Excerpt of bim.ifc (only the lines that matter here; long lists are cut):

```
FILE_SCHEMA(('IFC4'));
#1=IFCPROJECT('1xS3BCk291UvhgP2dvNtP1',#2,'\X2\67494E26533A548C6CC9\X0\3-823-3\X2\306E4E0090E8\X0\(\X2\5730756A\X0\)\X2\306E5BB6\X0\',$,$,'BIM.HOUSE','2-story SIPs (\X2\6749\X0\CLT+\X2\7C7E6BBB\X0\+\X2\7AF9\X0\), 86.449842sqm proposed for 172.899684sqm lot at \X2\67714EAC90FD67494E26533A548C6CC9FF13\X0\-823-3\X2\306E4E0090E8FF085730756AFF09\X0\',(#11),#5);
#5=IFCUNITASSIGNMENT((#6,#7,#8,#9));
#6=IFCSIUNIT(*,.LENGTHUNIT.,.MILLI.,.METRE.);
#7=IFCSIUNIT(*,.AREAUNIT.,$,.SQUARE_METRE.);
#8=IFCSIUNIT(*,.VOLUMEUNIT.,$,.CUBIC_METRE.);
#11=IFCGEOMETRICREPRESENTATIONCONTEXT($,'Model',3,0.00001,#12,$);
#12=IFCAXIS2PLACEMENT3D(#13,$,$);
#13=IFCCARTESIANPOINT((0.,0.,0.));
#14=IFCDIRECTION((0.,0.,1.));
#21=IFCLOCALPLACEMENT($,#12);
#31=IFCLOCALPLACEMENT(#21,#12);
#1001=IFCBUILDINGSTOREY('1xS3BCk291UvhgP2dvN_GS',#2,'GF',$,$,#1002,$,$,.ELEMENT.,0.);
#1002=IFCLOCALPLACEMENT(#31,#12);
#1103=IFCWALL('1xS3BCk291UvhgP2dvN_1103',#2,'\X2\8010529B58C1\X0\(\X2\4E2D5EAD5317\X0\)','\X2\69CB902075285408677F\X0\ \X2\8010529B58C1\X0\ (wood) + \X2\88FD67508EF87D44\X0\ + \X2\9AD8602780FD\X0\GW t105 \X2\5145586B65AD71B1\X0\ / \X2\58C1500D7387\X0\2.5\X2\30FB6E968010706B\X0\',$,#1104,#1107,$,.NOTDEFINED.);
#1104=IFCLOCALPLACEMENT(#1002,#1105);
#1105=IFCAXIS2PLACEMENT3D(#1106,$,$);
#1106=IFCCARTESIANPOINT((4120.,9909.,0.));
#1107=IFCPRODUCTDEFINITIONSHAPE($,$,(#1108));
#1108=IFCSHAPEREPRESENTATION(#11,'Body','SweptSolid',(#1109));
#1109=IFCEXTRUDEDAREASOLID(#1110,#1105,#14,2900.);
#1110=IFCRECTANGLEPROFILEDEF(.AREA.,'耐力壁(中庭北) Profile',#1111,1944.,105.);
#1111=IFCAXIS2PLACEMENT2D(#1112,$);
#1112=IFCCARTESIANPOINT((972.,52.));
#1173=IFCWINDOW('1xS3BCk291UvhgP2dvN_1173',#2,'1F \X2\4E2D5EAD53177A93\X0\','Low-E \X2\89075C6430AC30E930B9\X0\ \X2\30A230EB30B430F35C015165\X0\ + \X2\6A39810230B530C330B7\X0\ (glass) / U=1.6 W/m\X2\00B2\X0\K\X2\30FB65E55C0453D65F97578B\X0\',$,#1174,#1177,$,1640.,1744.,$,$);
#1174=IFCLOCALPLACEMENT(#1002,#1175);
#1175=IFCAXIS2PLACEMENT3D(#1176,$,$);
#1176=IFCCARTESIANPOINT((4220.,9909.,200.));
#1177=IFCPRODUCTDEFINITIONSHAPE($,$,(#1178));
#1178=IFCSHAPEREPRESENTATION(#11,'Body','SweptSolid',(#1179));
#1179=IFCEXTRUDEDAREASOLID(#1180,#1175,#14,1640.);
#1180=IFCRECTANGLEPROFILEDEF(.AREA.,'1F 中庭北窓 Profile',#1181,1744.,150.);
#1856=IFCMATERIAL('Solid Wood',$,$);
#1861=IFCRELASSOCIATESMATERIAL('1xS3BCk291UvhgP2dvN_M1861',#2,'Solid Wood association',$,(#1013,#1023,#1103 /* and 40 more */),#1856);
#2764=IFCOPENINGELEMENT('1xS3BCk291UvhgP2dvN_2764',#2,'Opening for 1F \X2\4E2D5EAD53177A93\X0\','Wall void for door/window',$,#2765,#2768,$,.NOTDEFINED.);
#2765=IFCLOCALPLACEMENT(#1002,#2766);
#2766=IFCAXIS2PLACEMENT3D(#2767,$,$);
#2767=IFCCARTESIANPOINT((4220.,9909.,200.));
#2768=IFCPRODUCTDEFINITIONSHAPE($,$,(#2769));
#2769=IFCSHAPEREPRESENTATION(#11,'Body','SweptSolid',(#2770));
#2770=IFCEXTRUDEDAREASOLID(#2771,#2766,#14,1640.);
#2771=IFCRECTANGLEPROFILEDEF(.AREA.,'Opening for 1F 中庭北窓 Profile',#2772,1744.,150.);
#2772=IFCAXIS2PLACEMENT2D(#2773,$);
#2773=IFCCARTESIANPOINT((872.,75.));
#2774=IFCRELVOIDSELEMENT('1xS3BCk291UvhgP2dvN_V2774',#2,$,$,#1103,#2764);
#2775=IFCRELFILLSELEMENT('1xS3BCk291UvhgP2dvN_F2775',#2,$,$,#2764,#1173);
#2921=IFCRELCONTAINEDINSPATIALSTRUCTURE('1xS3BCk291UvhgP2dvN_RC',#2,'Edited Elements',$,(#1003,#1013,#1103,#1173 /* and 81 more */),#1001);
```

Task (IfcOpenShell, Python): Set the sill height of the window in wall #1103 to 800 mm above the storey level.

```python
import numpy as np
import ifcopenshell
import ifcopenshell.api.geometry
import ifcopenshell.geom
import ifcopenshell.util.element
import ifcopenshell.util.placement
import ifcopenshell.util.shape
import ifcopenshell.util.unit

model = ifcopenshell.open("bim.ifc")
unit_scale = ifcopenshell.util.unit.calculate_unit_scale(model)

window = model.by_guid("1xS3BCk291UvhgP2dvN_1173")
opening = window.FillsVoids[0].RelatingOpeningElement
storey = ifcopenshell.util.element.get_container(window, ifc_class="IfcBuildingStorey")
level = ifcopenshell.util.placement.get_local_placement(storey.ObjectPlacement)[2, 3]

# The opening's origin need not be at the sill, so measure its lowest point.
shape = ifcopenshell.geom.create_shape(ifcopenshell.geom.settings(), opening)
bottom = ifcopenshell.util.shape.get_shape_bottom_elevation(shape, shape.geometry) / unit_scale
dz = level + 0.8 / unit_scale - bottom

shift = np.array([0.0, 0.0, dz])
# The window is not placed relative to its opening, so move both.
for product in (opening, window):
    matrix = ifcopenshell.util.placement.get_local_placement(product.ObjectPlacement)
    matrix[:3, 3] += shift
    ifcopenshell.api.geometry.edit_object_placement(model, product=product, matrix=matrix, is_si=False)

print(f"moved by {dz * unit_scale:+.3f} m")

model.write("bim_v2.ifc")
```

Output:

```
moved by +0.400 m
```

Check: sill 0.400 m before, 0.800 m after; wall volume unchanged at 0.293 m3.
